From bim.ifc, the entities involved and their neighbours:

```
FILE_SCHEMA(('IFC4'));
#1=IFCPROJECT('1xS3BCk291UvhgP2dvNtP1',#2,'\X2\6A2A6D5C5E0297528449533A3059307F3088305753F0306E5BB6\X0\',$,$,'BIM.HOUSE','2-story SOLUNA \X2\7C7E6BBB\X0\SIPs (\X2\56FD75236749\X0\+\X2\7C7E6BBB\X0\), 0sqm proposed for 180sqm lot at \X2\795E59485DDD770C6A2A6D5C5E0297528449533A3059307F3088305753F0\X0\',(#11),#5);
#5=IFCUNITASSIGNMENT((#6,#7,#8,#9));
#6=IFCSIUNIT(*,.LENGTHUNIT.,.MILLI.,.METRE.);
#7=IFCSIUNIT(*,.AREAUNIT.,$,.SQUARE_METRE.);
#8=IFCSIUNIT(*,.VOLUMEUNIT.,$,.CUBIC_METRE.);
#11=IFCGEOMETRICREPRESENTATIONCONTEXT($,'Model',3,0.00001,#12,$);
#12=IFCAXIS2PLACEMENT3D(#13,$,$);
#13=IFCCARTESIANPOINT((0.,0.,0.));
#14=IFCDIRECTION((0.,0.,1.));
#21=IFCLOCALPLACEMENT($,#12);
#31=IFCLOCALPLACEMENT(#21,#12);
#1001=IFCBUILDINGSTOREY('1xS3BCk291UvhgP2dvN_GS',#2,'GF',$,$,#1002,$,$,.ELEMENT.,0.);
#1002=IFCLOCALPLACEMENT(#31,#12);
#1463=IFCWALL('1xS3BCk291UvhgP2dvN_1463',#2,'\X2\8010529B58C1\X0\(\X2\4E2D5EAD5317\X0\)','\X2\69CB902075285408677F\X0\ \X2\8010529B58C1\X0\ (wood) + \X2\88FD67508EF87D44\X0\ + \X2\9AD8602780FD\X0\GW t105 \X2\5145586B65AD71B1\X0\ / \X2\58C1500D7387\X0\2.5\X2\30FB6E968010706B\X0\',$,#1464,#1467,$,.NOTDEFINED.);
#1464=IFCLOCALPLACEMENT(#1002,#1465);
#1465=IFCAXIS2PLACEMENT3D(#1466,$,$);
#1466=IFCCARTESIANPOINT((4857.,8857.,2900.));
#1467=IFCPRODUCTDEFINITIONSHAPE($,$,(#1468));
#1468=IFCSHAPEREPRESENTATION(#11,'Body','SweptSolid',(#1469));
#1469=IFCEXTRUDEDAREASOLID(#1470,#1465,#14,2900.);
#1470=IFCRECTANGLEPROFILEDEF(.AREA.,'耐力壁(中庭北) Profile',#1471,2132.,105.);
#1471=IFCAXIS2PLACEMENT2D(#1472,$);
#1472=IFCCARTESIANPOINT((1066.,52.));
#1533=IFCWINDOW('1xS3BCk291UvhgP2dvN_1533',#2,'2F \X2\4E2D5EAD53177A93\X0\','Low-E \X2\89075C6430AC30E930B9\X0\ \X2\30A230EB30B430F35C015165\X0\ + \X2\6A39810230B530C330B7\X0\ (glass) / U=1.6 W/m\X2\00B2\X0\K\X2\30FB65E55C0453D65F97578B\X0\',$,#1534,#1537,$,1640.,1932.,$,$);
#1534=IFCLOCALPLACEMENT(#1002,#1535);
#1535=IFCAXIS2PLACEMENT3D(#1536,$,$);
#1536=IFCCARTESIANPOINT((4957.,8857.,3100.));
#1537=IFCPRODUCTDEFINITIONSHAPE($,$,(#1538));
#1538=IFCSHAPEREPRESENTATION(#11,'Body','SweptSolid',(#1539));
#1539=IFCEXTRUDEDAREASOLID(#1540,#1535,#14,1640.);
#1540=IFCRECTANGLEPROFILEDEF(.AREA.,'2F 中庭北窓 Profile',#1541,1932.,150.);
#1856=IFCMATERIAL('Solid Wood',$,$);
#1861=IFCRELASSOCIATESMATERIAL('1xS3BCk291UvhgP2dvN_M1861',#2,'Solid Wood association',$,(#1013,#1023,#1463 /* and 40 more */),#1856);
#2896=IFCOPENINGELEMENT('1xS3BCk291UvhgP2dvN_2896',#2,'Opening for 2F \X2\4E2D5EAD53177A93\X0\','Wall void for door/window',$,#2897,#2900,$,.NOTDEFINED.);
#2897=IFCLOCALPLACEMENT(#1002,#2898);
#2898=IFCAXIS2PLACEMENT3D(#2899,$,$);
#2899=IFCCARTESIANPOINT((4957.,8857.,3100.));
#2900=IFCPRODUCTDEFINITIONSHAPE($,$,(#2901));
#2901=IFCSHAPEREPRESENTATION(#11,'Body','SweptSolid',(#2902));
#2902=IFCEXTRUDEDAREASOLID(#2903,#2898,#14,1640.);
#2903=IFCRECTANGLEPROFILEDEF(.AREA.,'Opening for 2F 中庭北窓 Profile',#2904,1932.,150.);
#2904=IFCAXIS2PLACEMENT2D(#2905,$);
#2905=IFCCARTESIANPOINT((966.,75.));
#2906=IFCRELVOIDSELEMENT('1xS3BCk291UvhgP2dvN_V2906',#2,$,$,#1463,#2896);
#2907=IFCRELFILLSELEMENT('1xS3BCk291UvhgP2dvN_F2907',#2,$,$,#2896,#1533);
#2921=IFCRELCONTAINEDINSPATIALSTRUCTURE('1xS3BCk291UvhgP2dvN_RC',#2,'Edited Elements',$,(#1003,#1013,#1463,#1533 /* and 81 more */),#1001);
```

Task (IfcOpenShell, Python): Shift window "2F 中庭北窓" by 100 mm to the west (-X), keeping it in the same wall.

```python
import ifcopenshell
import ifcopenshell.api.geometry
import ifcopenshell.util.placement
import ifcopenshell.util.unit

model = ifcopenshell.open("bim.ifc")
unit_scale = ifcopenshell.util.unit.calculate_unit_scale(model)

window = model.by_guid("1xS3BCk291UvhgP2dvN_1533")
opening = window.FillsVoids[0].RelatingOpeningElement
wall = opening.VoidsElements[0].RelatingBuildingElement

wall_matrix = ifcopenshell.util.placement.get_local_placement(wall.ObjectPlacement)
shift = wall_matrix[:3, 0] * -0.1 / unit_scale
before = ifcopenshell.util.placement.get_local_placement(window.ObjectPlacement)[:3, 3].copy()

# The window is not placed relative to its opening, so move both.
for product in (opening, window):
    matrix = ifcopenshell.util.placement.get_local_placement(product.ObjectPlacement)
    matrix[:3, 3] += shift
    ifcopenshell.api.geometry.edit_object_placement(model, product=product, matrix=matrix, is_si=False)

after = ifcopenshell.util.placement.get_local_placement(window.ObjectPlacement)[:3, 3]
print("window moved by", (after - before).round(3) + 0.0)

model.write("bim_updated.ifc")
```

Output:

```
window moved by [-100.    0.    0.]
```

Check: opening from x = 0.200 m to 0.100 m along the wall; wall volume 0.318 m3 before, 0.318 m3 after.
